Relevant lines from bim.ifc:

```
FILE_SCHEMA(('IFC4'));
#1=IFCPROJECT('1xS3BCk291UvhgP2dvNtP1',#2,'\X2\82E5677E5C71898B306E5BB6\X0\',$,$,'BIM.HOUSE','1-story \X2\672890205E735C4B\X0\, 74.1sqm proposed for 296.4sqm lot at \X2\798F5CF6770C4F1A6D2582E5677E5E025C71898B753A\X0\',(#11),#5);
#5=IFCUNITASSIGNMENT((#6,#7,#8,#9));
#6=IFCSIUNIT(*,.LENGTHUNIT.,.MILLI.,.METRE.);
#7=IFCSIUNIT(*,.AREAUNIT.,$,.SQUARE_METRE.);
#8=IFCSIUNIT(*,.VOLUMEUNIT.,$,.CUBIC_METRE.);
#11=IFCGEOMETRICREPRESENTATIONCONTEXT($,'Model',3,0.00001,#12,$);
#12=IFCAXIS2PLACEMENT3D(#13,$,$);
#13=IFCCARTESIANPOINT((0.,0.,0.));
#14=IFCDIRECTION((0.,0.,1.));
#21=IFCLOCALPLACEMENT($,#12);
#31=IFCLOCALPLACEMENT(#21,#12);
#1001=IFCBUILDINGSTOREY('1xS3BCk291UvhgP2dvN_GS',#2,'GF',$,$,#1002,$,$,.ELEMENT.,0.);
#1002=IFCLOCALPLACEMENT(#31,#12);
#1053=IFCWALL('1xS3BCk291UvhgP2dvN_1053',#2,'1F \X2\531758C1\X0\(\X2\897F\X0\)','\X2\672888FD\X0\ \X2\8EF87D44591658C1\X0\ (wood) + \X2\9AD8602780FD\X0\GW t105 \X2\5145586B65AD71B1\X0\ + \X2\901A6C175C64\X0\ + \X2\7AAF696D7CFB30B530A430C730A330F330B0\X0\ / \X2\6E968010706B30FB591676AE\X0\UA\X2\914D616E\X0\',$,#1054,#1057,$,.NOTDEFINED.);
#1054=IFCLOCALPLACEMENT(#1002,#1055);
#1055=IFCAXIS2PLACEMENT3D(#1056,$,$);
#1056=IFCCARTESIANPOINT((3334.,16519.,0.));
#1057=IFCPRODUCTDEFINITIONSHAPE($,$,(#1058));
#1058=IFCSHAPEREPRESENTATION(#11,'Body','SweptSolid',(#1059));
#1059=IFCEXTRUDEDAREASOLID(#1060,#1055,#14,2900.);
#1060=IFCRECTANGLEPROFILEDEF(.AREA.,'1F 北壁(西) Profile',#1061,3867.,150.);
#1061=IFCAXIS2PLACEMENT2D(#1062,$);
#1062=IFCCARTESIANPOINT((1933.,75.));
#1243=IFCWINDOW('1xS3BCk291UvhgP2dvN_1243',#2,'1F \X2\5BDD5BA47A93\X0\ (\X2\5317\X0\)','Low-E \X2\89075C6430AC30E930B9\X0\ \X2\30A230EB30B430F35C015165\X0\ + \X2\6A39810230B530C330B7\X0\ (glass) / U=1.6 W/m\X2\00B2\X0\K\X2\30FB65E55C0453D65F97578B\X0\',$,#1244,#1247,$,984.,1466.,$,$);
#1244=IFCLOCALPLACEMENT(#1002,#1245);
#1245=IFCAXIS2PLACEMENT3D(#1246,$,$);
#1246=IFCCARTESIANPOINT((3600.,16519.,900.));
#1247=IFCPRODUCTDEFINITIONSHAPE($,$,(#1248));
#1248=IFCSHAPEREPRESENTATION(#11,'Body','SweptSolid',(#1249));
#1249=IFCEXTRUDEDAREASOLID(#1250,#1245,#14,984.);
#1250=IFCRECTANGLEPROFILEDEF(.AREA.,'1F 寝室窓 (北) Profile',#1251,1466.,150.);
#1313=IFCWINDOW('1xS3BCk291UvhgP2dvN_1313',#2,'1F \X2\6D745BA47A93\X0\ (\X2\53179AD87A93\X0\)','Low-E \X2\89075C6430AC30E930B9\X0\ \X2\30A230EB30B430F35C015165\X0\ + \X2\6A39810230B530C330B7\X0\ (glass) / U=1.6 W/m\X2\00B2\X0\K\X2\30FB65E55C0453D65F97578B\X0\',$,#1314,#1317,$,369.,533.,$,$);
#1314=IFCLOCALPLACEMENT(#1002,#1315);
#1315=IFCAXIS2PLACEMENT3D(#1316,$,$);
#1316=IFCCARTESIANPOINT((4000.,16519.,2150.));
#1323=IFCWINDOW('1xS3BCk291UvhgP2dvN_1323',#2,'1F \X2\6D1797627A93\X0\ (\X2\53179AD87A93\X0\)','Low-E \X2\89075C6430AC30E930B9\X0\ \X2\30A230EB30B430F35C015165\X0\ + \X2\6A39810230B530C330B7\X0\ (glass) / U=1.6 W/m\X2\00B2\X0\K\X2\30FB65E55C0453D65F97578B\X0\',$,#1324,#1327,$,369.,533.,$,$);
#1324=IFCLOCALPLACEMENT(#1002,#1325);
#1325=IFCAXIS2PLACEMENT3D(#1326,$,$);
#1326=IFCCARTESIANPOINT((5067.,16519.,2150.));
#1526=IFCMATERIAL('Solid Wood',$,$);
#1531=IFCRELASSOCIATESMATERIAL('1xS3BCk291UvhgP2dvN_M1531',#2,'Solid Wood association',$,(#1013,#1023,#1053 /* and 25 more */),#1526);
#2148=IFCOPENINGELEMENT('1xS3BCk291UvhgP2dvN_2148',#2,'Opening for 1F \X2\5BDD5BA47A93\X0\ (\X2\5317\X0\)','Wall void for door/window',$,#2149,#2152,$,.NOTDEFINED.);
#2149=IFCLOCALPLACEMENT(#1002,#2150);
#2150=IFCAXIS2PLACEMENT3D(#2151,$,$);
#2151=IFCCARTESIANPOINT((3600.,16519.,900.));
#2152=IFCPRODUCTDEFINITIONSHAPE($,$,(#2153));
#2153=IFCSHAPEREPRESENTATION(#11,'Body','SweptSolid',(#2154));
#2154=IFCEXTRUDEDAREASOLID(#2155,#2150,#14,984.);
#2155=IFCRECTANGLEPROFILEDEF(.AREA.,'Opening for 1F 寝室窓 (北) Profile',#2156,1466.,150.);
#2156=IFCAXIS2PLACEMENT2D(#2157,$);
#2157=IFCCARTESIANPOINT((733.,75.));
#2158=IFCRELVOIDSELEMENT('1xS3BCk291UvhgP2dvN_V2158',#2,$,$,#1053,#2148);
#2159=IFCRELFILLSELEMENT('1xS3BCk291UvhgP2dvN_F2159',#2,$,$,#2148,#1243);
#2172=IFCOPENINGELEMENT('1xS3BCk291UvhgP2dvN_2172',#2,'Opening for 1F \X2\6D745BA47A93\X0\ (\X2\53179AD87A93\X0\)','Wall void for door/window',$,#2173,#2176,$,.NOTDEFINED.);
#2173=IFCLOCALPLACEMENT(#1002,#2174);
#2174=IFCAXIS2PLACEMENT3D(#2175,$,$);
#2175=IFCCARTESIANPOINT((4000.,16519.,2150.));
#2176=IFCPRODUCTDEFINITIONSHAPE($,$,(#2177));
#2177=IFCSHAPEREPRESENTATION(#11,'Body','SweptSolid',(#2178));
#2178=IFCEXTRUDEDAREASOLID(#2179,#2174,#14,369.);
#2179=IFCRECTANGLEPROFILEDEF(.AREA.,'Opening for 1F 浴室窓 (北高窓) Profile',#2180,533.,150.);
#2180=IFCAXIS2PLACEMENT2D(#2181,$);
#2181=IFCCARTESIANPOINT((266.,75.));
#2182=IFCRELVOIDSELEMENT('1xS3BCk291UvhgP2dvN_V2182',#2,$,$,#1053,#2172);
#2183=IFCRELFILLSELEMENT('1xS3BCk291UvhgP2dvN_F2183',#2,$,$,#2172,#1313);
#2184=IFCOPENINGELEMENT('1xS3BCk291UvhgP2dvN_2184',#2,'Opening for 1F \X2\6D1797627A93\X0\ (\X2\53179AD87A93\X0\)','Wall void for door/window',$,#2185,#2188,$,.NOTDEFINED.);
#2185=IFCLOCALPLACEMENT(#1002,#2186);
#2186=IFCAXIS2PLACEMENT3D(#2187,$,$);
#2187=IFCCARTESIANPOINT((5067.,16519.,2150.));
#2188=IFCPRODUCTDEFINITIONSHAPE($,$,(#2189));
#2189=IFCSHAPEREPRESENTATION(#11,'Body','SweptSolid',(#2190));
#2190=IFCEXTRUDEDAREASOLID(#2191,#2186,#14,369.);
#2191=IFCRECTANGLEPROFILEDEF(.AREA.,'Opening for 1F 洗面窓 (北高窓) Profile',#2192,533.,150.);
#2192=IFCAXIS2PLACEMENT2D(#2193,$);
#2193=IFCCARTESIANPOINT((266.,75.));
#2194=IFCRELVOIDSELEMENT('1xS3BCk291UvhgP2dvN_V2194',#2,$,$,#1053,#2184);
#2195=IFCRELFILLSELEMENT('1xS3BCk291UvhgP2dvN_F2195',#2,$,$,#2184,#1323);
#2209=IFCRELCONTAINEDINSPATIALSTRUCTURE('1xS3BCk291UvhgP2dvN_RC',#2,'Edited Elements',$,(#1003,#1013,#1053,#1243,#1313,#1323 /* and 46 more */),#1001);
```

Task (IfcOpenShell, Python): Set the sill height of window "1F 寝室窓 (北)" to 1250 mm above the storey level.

```python
import numpy as np
import ifcopenshell
import ifcopenshell.api.geometry
import ifcopenshell.geom
import ifcopenshell.util.element
import ifcopenshell.util.placement
import ifcopenshell.util.shape
import ifcopenshell.util.unit

model = ifcopenshell.open("bim.ifc")
unit_scale = ifcopenshell.util.unit.calculate_unit_scale(model)

window = model.by_guid("1xS3BCk291UvhgP2dvN_1243")
opening = window.FillsVoids[0].RelatingOpeningElement
storey = ifcopenshell.util.element.get_container(window, ifc_class="IfcBuildingStorey")
level = ifcopenshell.util.placement.get_local_placement(storey.ObjectPlacement)[2, 3]

# The opening's origin need not be at the sill, so measure its lowest point.
shape = ifcopenshell.geom.create_shape(ifcopenshell.geom.settings(), opening)
bottom = ifcopenshell.util.shape.get_shape_bottom_elevation(shape, shape.geometry) / unit_scale
dz = level + 1250.0 - bottom

shift = np.array([0.0, 0.0, dz])
# The window is not placed relative to its opening, so move both.
for product in (opening, window):
    matrix = ifcopenshell.util.placement.get_local_placement(product.ObjectPlacement)
    matrix[:3, 3] += shift
    ifcopenshell.api.geometry.edit_object_placement(model, product=product, matrix=matrix, is_si=False)

print(f"moved by {dz * unit_scale:+.3f} m")

model.write("bim_v2.ifc")
```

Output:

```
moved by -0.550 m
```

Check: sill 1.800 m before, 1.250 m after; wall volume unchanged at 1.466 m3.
